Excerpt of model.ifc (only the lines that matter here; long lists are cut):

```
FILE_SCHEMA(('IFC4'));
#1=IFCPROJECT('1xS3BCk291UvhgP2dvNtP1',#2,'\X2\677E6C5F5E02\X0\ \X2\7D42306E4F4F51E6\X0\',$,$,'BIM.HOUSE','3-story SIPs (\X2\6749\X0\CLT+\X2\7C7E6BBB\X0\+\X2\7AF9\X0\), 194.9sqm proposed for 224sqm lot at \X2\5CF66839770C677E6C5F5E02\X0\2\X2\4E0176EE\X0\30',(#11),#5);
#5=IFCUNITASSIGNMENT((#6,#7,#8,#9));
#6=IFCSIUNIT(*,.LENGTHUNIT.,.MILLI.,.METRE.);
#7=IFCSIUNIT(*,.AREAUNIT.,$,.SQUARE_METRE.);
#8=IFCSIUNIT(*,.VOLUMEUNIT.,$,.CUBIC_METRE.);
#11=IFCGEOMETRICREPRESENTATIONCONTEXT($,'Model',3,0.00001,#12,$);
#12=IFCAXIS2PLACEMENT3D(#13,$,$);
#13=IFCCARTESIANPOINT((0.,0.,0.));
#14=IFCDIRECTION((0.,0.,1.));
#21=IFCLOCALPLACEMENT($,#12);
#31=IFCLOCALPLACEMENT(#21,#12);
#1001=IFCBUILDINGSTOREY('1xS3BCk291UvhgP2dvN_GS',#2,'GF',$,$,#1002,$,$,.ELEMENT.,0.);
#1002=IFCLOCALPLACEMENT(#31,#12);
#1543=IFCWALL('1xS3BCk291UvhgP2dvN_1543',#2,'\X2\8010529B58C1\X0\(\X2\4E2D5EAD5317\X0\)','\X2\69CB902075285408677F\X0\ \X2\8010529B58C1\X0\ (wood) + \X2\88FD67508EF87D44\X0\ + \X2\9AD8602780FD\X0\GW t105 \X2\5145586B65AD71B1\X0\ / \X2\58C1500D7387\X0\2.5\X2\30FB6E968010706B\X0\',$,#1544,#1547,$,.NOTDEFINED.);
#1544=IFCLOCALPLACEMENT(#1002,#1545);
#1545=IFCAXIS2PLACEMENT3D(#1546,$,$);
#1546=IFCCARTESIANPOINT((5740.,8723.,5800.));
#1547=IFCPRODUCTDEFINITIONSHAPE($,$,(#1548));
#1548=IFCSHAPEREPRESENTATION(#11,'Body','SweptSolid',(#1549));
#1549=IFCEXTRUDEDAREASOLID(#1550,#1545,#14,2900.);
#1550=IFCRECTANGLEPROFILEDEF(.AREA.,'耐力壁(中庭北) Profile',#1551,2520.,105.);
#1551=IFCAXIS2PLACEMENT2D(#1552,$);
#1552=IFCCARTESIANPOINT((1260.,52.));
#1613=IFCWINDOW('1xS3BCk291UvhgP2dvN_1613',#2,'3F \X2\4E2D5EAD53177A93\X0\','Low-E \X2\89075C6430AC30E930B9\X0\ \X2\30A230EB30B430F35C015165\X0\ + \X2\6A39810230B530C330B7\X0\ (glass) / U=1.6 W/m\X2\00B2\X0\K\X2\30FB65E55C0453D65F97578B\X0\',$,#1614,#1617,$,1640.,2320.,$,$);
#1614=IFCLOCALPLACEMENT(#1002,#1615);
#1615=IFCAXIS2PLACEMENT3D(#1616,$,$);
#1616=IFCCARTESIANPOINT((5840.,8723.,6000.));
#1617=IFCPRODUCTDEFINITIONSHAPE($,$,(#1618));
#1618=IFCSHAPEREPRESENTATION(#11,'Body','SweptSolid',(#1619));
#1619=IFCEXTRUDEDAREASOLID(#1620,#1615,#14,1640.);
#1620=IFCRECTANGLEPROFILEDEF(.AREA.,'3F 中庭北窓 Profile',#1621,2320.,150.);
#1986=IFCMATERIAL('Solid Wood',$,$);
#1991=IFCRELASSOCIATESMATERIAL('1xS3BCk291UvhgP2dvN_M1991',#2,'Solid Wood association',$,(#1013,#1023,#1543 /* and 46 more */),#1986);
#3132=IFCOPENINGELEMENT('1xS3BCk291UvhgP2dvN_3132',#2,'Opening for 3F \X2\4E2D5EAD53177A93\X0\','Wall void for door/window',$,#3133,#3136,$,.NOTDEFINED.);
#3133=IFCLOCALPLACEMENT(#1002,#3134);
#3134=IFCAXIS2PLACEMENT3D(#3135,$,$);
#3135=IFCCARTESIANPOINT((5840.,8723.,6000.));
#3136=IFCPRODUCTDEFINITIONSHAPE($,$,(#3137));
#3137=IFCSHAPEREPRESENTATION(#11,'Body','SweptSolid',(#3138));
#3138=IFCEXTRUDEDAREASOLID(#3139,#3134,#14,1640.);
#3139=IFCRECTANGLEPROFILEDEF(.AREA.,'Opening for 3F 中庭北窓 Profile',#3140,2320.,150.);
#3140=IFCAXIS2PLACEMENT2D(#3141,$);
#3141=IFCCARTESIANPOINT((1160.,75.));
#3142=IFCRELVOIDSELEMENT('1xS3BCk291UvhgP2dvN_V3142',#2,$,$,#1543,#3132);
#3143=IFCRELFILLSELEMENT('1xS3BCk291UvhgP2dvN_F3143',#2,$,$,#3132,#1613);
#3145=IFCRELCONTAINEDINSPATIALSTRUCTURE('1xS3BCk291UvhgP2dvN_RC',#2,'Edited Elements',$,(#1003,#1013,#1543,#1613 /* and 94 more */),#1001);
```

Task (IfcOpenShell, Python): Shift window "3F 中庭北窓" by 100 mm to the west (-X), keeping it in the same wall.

```python
import ifcopenshell
import ifcopenshell.api.geometry
import ifcopenshell.util.placement

model = ifcopenshell.open("model.ifc")

window = model.by_guid("1xS3BCk291UvhgP2dvN_1613")
opening = window.FillsVoids[0].RelatingOpeningElement
wall = opening.VoidsElements[0].RelatingBuildingElement

wall_matrix = ifcopenshell.util.placement.get_local_placement(wall.ObjectPlacement)
shift = wall_matrix[:3, 0] * -100.0
before = ifcopenshell.util.placement.get_local_placement(window.ObjectPlacement)[:3, 3].copy()

# The window is not placed relative to its opening, so move both.
for product in (opening, window):
    matrix = ifcopenshell.util.placement.get_local_placement(product.ObjectPlacement)
    matrix[:3, 3] += shift
    ifcopenshell.api.geometry.edit_object_placement(model, product=product, matrix=matrix, is_si=False)

after = ifcopenshell.util.placement.get_local_placement(window.ObjectPlacement)[:3, 3]
print("window moved by", (after - before).round(3) + 0.0)

model.write("model-out.ifc")
```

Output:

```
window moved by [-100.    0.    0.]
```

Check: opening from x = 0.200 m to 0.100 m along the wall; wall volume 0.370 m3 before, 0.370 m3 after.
